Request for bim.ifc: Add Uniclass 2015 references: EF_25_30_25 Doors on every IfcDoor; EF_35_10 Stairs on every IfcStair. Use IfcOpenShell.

First a look at what the model holds.

```python
import ifcopenshell

model = ifcopenshell.open("bim.ifc")
print(model.schema)
print("classifications:", [c.Name for c in model.by_type("IfcClassification")])
for ifc_class in ("IfcDoor", "IfcRoof", "IfcStair", "IfcWall", "IfcWindow"):
    print(ifc_class, len(model.by_type(ifc_class)))
```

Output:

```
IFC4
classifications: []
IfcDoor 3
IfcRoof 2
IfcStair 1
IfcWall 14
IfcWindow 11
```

```python
import ifcopenshell
import ifcopenshell.api.classification

model = ifcopenshell.open("bim.ifc")

system = ifcopenshell.api.classification.add_classification(model, classification="Uniclass 2015")

codes = {
    "IfcDoor": ("EF_25_30_25", "Doors"),
    "IfcStair": ("EF_35_10", "Stairs"),
}
for ifc_class, (code, name) in codes.items():
    products = model.by_type(ifc_class)
    ifcopenshell.api.classification.add_reference(
        model, products=products, classification=system, identification=code, name=name
    )
    print(code, len(products))

model.write("bim_edited.ifc")
```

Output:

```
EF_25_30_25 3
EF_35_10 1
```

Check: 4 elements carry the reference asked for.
